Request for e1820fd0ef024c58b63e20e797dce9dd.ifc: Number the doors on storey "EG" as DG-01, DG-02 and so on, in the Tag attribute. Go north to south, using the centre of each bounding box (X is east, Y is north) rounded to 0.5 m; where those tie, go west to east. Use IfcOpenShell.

First a look at what the model holds.

```python
import ifcopenshell
import ifcopenshell.util.element
import ifcopenshell.util.placement

model = ifcopenshell.open("e1820fd0ef024c58b63e20e797dce9dd.ifc")
print(model.schema)
storey = next(s for s in model.by_type("IfcBuildingStorey") if s.Name == "EG")
doors = [e for e in ifcopenshell.util.element.get_decomposition(storey) if e.is_a("IfcDoor")]
for e in sorted(doors, key=lambda e: e.id()):
    origin = ifcopenshell.util.placement.get_local_placement(e.ObjectPlacement)[:3, 3]
    print(e.id(), e.Tag, e.Name, origin.round(2) + 0.0, sep=" | ")
```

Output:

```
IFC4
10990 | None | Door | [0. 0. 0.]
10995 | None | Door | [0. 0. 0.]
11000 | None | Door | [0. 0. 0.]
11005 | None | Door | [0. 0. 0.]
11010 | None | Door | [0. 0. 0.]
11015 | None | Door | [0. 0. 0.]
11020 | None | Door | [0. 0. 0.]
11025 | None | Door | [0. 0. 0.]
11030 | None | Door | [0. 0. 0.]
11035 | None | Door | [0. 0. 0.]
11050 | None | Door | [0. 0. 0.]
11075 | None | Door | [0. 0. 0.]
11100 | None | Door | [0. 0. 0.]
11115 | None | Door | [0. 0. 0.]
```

```python
import ifcopenshell
import ifcopenshell.geom
import ifcopenshell.util.element
import ifcopenshell.util.shape

model = ifcopenshell.open("e1820fd0ef024c58b63e20e797dce9dd.ifc")
settings = ifcopenshell.geom.settings()
settings.set("use-world-coords", True)


def centre(element):
    shape = ifcopenshell.geom.create_shape(settings, element)
    return ifcopenshell.util.shape.get_bbox_centroid(shape.geometry)


storey = next(s for s in model.by_type("IfcBuildingStorey") if s.Name == "EG")
doors = [e for e in ifcopenshell.util.element.get_decomposition(storey) if e.is_a("IfcDoor")]

# Insertion points can sit at a corner or the storey origin, so sort by the geometry (in metres).
centres = {e: centre(e) for e in doors}
doors.sort(key=lambda e: (-round(centres[e][1] / 0.5), centres[e][0]))

for i, e in enumerate(doors, start=1):
    number = f"DG-{i:02d}"
    e.Tag = number
    print(e.id(), number)

model.write("e1820fd0ef024c58b63e20e797dce9dd_rev.ifc")
```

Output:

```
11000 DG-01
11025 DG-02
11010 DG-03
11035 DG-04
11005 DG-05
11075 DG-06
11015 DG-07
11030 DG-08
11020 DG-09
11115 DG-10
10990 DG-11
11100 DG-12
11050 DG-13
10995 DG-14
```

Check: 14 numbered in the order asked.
